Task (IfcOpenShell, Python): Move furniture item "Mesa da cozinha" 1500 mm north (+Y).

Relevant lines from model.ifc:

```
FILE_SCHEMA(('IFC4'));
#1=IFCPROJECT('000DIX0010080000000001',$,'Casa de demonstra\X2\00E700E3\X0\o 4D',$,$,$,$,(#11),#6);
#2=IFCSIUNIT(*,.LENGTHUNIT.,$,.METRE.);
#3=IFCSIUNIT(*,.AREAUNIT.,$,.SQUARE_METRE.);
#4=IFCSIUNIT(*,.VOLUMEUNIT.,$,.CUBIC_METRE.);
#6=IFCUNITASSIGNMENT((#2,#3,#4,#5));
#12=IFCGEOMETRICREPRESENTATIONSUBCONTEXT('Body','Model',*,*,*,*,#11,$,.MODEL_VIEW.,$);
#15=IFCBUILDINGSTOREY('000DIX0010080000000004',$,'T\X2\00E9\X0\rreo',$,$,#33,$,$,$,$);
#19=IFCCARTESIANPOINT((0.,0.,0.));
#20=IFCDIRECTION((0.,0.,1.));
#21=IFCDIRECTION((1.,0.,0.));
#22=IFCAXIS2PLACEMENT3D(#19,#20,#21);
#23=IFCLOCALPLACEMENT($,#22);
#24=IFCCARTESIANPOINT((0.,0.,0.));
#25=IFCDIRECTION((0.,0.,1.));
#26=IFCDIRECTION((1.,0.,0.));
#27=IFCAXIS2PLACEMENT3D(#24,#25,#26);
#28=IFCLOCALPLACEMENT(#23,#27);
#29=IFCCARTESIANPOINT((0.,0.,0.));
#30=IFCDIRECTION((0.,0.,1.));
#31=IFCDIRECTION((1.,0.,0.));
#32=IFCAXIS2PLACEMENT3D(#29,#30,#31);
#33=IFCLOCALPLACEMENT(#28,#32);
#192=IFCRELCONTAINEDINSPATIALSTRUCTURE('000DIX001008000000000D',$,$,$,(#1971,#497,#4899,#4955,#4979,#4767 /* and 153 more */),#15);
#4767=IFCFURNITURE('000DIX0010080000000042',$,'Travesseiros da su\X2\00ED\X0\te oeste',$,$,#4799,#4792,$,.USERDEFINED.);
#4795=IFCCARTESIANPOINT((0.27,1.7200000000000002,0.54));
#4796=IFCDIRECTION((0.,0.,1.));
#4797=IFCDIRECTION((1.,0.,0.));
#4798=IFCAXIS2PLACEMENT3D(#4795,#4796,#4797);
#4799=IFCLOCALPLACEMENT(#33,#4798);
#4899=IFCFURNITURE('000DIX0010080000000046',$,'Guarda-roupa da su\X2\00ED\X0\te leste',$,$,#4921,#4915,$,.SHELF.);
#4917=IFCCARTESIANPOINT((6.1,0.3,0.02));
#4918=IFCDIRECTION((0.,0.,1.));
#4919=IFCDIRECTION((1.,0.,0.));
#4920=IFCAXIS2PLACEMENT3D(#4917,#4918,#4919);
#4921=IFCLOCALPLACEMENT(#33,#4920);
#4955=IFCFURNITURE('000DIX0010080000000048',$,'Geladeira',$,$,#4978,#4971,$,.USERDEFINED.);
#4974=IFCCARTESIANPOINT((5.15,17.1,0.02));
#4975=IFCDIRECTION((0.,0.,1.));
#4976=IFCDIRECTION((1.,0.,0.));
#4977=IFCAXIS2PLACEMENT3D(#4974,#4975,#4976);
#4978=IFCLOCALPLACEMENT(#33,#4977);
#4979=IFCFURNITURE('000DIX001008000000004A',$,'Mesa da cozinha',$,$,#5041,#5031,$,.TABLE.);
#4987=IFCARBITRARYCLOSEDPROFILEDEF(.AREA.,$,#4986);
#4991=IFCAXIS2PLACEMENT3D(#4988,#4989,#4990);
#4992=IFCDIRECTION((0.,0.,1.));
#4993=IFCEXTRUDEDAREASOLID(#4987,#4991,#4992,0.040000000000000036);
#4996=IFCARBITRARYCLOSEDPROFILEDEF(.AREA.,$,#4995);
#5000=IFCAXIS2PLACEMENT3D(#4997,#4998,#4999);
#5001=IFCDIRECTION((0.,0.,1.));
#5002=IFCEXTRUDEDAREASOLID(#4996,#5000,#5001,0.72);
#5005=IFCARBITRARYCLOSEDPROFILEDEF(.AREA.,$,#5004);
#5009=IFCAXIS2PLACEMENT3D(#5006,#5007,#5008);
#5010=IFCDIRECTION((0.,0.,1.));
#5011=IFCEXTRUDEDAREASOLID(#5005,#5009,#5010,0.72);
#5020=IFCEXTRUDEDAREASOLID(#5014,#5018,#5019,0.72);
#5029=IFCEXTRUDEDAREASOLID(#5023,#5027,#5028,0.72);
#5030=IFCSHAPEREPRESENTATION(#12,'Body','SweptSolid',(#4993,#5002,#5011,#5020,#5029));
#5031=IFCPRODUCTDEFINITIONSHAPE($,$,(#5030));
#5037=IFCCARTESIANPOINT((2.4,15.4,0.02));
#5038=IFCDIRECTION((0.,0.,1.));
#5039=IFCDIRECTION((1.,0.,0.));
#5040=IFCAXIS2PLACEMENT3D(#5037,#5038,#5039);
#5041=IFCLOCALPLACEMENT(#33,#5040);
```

```python
import ifcopenshell
import ifcopenshell.api.geometry
import ifcopenshell.util.placement

model = ifcopenshell.open("model.ifc")

item = model.by_guid("000DIX001008000000004A")
matrix = ifcopenshell.util.placement.get_local_placement(item.ObjectPlacement)
matrix[1, 3] += 1.5
ifcopenshell.api.geometry.edit_object_placement(model, product=item, matrix=matrix, is_si=False)

print(ifcopenshell.util.placement.get_local_placement(item.ObjectPlacement).round(3) + 0.0)

model.write("model_rev.ifc")
```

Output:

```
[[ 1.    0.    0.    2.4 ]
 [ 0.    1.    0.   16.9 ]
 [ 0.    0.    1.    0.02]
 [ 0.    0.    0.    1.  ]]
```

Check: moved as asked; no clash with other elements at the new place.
